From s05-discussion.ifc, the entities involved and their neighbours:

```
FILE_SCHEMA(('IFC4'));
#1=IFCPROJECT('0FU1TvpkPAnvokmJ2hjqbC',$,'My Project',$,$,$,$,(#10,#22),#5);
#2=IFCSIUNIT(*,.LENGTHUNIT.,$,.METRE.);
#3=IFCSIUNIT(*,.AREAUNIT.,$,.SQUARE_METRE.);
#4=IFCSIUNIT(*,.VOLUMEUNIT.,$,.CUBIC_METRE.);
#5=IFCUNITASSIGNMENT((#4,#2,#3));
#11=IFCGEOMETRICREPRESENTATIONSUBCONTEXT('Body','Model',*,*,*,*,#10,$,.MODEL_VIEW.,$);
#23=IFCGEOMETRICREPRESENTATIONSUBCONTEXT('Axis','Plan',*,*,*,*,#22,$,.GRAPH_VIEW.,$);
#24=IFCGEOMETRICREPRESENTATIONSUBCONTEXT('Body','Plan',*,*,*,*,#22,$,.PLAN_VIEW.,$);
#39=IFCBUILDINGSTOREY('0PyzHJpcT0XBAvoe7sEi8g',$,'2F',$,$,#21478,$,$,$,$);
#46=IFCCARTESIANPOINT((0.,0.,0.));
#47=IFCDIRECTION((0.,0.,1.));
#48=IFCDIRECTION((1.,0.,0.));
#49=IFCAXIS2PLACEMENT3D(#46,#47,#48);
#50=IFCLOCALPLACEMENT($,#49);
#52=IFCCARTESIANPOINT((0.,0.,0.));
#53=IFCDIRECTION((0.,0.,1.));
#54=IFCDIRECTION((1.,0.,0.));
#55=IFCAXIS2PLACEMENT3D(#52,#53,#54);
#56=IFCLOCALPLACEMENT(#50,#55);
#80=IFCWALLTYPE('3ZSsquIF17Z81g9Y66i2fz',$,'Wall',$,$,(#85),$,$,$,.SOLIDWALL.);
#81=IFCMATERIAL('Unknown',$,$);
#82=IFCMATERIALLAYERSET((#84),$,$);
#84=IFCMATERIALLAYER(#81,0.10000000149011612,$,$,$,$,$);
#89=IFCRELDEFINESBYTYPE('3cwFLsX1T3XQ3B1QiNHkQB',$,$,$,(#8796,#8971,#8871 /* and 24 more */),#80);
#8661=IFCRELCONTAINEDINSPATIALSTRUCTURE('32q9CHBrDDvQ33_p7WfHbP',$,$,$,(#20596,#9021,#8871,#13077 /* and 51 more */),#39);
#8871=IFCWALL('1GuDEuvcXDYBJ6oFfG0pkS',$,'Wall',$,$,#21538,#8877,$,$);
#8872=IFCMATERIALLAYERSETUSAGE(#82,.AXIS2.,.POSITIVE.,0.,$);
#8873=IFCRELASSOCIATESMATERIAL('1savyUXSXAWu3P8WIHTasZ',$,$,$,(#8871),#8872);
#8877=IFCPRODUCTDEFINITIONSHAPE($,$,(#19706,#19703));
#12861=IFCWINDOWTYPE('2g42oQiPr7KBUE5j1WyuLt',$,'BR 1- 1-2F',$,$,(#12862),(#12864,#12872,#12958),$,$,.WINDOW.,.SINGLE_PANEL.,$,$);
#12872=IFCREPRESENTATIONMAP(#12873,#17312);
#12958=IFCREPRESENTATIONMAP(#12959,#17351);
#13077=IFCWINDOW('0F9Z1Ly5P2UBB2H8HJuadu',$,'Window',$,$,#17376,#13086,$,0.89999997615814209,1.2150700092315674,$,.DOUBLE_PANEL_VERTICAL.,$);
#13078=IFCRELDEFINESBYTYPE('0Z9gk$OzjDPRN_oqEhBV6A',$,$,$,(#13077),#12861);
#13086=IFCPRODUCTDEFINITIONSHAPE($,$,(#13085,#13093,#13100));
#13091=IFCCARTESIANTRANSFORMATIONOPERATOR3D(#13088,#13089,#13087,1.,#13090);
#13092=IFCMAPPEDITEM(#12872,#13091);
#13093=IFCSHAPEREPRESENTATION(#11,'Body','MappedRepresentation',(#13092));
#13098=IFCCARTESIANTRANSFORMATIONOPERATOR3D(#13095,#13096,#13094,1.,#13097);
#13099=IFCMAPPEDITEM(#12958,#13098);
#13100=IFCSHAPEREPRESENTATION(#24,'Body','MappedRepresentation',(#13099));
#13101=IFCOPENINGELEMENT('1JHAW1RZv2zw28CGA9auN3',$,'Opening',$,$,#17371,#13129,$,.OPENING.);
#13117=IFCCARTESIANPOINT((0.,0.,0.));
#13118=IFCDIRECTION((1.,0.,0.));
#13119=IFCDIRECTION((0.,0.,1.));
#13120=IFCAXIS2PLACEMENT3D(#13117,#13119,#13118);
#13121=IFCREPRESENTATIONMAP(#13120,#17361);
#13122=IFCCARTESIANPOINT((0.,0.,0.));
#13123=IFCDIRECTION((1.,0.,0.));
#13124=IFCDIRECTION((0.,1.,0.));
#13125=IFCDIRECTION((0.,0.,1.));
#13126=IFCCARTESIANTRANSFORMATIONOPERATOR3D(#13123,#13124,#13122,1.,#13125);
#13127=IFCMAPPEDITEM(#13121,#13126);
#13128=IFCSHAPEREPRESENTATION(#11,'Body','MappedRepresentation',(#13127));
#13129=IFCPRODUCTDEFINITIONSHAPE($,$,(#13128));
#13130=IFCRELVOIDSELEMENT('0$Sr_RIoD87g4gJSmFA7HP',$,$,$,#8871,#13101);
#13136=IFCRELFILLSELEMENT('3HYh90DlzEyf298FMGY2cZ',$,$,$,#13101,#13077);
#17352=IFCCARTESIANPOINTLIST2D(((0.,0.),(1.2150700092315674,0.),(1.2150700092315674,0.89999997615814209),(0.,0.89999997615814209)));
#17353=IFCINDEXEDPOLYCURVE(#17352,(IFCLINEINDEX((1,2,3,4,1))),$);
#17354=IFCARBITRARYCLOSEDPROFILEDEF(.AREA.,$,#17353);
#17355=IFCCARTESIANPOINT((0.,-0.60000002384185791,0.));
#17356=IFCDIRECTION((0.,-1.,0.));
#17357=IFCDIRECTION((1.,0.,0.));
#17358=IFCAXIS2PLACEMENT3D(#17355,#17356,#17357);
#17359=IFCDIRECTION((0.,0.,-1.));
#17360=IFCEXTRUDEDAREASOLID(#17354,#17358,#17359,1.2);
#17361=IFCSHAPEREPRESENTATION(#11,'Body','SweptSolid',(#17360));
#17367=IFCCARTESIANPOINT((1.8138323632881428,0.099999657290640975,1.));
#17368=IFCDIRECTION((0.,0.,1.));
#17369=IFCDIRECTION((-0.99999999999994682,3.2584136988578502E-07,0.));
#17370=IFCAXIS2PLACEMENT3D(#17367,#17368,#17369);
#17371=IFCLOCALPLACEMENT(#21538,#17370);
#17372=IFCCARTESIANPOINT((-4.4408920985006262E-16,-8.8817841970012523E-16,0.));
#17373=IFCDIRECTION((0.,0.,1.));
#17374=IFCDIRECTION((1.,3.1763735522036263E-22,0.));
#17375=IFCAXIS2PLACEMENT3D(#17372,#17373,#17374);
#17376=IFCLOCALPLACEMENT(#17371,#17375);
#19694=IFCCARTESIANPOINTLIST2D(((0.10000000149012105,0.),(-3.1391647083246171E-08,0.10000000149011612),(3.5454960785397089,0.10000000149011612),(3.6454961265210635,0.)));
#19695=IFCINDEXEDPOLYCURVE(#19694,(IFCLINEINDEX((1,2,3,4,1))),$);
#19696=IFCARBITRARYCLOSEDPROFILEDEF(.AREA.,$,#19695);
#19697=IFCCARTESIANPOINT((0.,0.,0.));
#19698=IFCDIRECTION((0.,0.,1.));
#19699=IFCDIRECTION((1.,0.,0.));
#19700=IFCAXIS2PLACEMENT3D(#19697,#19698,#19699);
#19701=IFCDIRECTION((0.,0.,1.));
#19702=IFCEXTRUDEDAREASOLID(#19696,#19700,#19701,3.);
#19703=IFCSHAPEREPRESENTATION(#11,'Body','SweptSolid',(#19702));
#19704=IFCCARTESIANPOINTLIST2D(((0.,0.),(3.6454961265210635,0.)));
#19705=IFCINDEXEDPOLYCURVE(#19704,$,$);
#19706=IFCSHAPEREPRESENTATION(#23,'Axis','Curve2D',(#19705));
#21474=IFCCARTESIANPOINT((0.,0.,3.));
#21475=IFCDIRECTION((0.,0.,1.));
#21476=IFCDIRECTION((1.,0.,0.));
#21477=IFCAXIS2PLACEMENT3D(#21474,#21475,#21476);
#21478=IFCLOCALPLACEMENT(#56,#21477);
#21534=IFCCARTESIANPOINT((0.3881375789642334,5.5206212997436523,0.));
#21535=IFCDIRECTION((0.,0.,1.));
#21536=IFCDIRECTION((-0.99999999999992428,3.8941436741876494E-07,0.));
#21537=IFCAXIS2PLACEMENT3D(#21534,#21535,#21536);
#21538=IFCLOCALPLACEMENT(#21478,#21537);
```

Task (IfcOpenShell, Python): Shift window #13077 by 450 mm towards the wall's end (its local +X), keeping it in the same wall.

```python
import ifcopenshell
import ifcopenshell.api.geometry
import ifcopenshell.util.placement

model = ifcopenshell.open("s05-discussion.ifc")

window = model.by_guid("0F9Z1Ly5P2UBB2H8HJuadu")
opening = window.FillsVoids[0].RelatingOpeningElement
wall = opening.VoidsElements[0].RelatingBuildingElement

wall_matrix = ifcopenshell.util.placement.get_local_placement(wall.ObjectPlacement)
shift = wall_matrix[:3, 0] * 0.45
before = ifcopenshell.util.placement.get_local_placement(window.ObjectPlacement)[:3, 3].copy()

# The window is placed relative to its opening, so it follows when the opening moves.
matrix = ifcopenshell.util.placement.get_local_placement(opening.ObjectPlacement)
matrix[:3, 3] += shift
ifcopenshell.api.geometry.edit_object_placement(
    model, product=opening, matrix=matrix, is_si=False, should_transform_children=True
)

after = ifcopenshell.util.placement.get_local_placement(window.ObjectPlacement)[:3, 3]
print("window moved by", (after - before).round(3) + 0.0)

model.write("s05-discussion_updated.ifc")
```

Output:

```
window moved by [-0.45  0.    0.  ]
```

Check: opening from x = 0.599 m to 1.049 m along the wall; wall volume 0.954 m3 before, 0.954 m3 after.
